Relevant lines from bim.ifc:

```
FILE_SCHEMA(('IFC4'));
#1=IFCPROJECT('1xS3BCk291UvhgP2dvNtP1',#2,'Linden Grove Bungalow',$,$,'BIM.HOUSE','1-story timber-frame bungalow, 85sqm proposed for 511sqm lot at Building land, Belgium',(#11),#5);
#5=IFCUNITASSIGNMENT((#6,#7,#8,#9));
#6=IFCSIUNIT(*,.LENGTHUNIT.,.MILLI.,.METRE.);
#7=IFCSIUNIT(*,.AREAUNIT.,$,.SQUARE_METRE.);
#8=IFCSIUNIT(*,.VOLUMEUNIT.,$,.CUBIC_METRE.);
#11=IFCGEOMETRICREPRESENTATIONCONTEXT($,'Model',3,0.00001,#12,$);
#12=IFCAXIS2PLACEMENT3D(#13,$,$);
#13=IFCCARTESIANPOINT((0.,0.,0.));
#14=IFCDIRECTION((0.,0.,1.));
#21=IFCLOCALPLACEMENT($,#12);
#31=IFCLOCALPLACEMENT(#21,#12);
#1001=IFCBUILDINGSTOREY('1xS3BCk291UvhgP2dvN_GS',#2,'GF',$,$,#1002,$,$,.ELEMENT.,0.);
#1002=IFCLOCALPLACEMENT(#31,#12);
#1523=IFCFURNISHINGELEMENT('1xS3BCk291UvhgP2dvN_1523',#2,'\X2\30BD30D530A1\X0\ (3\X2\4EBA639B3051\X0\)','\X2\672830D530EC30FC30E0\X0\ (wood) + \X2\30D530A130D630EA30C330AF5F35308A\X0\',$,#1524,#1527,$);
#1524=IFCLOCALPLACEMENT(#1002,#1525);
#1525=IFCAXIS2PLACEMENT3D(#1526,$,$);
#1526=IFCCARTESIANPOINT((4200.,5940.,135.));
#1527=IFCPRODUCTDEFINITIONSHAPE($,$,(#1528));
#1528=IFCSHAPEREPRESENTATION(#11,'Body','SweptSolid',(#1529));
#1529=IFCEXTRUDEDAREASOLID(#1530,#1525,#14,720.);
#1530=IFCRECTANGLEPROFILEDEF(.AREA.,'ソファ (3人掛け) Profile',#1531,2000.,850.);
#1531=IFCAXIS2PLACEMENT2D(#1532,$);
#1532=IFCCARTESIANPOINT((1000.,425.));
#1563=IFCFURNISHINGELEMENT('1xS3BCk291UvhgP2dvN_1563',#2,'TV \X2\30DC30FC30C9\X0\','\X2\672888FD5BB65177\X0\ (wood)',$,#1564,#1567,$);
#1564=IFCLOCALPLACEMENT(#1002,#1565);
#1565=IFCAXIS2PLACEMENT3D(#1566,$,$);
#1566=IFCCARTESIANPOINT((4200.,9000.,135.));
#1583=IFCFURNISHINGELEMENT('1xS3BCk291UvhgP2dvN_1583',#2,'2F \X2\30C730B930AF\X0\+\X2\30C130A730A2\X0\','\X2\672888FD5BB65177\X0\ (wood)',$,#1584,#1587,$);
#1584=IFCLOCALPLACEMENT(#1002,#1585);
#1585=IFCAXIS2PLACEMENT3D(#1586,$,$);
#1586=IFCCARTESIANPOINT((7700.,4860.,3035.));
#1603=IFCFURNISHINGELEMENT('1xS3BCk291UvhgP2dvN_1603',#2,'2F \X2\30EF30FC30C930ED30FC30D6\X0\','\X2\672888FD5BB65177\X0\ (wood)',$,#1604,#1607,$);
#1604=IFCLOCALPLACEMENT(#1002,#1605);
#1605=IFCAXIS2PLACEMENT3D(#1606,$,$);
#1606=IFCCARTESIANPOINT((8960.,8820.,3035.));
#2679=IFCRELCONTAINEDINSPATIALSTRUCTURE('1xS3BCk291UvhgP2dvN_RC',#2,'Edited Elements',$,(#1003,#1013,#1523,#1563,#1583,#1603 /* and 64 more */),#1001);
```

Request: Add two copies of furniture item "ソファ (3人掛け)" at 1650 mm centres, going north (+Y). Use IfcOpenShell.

```python
import numpy as np
import ifcopenshell
import ifcopenshell.api.geometry
import ifcopenshell.api.root
import ifcopenshell.util.element
import ifcopenshell.util.placement
import ifcopenshell.util.unit

model = ifcopenshell.open("bim.ifc")
unit_scale = ifcopenshell.util.unit.calculate_unit_scale(model)


def reuse_history(source, copy):
    """copy_class also copies each property set's owner history, people and application; keep the originals."""
    for rel in copy.IsDefinedBy:
        if rel.is_a("IfcRelDefinesByProperties") and (history := rel.RelatingPropertyDefinition.OwnerHistory):
            rel.RelatingPropertyDefinition.OwnerHistory = source.OwnerHistory
            ifcopenshell.util.element.remove_deep2(model, history)


source = model.by_id(1523)
base = ifcopenshell.util.placement.get_local_placement(source.ObjectPlacement)
step = np.array([0.0, 1.0, 0.0]) * 1.65 / unit_scale

for i in range(1, 3):
    copy = ifcopenshell.api.root.copy_class(model, product=source)
    copy.Representation = ifcopenshell.util.element.copy_deep(
        model, source.Representation, exclude=["IfcGeometricRepresentationContext", "IfcRepresentationMap"]
    )
    reuse_history(source, copy)
    matrix = base.copy()
    matrix[:3, 3] += i * step
    print("added at", matrix[:3, 3].round(3) + 0.0)
    ifcopenshell.api.geometry.edit_object_placement(model, product=copy, matrix=matrix, is_si=False)

model.write("bim_updated.ifc")
```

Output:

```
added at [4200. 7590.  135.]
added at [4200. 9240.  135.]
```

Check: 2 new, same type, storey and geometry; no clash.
